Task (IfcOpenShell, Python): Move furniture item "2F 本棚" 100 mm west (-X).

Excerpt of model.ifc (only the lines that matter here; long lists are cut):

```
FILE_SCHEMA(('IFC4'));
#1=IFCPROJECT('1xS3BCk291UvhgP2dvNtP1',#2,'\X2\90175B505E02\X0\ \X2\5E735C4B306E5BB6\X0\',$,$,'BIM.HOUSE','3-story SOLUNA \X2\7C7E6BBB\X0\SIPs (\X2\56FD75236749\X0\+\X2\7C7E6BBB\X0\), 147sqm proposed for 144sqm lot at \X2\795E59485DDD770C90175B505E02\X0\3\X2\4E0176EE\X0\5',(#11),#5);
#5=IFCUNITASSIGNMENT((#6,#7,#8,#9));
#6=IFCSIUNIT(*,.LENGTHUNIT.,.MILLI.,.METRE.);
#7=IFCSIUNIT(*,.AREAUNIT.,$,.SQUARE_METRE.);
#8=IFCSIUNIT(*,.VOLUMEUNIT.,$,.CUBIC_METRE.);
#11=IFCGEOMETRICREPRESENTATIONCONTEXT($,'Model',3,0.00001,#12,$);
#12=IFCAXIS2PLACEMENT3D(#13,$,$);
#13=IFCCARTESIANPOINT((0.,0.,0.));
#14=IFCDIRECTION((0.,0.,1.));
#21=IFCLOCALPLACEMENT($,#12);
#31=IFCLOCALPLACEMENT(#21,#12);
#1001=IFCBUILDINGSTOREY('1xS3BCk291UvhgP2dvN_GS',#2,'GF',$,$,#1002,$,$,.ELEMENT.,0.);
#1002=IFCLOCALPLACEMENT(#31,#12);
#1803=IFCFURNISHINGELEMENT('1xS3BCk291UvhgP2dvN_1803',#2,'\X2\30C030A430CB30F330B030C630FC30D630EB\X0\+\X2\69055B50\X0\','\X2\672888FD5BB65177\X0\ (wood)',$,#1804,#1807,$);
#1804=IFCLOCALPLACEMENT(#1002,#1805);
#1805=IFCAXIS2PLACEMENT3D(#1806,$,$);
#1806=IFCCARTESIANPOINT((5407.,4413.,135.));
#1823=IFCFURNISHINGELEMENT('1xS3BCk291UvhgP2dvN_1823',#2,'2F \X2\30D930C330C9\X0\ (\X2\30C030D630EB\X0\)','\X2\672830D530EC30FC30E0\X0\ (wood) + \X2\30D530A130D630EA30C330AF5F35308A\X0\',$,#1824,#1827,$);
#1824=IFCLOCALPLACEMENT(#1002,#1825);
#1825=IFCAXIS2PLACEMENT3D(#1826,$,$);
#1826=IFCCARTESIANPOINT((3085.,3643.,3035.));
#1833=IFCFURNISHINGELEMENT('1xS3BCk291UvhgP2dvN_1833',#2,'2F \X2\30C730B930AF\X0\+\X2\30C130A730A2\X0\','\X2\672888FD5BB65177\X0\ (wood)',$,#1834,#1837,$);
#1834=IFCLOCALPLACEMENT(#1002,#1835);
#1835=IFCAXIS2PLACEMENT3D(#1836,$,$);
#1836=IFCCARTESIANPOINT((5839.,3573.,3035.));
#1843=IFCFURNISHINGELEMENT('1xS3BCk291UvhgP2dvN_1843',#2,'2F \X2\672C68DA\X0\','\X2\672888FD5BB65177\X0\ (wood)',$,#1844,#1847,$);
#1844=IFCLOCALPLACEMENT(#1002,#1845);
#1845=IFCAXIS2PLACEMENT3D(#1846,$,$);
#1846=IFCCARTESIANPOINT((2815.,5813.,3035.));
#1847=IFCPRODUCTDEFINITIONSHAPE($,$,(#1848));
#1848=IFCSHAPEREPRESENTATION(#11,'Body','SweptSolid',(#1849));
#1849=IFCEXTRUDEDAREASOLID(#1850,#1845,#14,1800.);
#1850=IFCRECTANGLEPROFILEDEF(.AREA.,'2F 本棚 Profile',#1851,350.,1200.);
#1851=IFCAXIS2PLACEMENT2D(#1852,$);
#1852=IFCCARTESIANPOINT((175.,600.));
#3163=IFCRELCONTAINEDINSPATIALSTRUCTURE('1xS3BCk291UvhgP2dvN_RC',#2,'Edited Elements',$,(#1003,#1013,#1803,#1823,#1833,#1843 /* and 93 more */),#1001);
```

```python
import ifcopenshell
import ifcopenshell.api.geometry
import ifcopenshell.util.placement
import ifcopenshell.util.unit

model = ifcopenshell.open("model.ifc")
unit_scale = ifcopenshell.util.unit.calculate_unit_scale(model)

item = model.by_guid("1xS3BCk291UvhgP2dvN_1843")
matrix = ifcopenshell.util.placement.get_local_placement(item.ObjectPlacement)
matrix[0, 3] -= 0.1 / unit_scale
ifcopenshell.api.geometry.edit_object_placement(model, product=item, matrix=matrix, is_si=False)

print(ifcopenshell.util.placement.get_local_placement(item.ObjectPlacement).round(3) + 0.0)

model.write("model_v2.ifc")
```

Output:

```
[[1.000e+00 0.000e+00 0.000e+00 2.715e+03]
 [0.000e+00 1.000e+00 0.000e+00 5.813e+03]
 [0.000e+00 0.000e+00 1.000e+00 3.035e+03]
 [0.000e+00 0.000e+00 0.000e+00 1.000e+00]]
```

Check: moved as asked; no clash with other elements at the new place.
